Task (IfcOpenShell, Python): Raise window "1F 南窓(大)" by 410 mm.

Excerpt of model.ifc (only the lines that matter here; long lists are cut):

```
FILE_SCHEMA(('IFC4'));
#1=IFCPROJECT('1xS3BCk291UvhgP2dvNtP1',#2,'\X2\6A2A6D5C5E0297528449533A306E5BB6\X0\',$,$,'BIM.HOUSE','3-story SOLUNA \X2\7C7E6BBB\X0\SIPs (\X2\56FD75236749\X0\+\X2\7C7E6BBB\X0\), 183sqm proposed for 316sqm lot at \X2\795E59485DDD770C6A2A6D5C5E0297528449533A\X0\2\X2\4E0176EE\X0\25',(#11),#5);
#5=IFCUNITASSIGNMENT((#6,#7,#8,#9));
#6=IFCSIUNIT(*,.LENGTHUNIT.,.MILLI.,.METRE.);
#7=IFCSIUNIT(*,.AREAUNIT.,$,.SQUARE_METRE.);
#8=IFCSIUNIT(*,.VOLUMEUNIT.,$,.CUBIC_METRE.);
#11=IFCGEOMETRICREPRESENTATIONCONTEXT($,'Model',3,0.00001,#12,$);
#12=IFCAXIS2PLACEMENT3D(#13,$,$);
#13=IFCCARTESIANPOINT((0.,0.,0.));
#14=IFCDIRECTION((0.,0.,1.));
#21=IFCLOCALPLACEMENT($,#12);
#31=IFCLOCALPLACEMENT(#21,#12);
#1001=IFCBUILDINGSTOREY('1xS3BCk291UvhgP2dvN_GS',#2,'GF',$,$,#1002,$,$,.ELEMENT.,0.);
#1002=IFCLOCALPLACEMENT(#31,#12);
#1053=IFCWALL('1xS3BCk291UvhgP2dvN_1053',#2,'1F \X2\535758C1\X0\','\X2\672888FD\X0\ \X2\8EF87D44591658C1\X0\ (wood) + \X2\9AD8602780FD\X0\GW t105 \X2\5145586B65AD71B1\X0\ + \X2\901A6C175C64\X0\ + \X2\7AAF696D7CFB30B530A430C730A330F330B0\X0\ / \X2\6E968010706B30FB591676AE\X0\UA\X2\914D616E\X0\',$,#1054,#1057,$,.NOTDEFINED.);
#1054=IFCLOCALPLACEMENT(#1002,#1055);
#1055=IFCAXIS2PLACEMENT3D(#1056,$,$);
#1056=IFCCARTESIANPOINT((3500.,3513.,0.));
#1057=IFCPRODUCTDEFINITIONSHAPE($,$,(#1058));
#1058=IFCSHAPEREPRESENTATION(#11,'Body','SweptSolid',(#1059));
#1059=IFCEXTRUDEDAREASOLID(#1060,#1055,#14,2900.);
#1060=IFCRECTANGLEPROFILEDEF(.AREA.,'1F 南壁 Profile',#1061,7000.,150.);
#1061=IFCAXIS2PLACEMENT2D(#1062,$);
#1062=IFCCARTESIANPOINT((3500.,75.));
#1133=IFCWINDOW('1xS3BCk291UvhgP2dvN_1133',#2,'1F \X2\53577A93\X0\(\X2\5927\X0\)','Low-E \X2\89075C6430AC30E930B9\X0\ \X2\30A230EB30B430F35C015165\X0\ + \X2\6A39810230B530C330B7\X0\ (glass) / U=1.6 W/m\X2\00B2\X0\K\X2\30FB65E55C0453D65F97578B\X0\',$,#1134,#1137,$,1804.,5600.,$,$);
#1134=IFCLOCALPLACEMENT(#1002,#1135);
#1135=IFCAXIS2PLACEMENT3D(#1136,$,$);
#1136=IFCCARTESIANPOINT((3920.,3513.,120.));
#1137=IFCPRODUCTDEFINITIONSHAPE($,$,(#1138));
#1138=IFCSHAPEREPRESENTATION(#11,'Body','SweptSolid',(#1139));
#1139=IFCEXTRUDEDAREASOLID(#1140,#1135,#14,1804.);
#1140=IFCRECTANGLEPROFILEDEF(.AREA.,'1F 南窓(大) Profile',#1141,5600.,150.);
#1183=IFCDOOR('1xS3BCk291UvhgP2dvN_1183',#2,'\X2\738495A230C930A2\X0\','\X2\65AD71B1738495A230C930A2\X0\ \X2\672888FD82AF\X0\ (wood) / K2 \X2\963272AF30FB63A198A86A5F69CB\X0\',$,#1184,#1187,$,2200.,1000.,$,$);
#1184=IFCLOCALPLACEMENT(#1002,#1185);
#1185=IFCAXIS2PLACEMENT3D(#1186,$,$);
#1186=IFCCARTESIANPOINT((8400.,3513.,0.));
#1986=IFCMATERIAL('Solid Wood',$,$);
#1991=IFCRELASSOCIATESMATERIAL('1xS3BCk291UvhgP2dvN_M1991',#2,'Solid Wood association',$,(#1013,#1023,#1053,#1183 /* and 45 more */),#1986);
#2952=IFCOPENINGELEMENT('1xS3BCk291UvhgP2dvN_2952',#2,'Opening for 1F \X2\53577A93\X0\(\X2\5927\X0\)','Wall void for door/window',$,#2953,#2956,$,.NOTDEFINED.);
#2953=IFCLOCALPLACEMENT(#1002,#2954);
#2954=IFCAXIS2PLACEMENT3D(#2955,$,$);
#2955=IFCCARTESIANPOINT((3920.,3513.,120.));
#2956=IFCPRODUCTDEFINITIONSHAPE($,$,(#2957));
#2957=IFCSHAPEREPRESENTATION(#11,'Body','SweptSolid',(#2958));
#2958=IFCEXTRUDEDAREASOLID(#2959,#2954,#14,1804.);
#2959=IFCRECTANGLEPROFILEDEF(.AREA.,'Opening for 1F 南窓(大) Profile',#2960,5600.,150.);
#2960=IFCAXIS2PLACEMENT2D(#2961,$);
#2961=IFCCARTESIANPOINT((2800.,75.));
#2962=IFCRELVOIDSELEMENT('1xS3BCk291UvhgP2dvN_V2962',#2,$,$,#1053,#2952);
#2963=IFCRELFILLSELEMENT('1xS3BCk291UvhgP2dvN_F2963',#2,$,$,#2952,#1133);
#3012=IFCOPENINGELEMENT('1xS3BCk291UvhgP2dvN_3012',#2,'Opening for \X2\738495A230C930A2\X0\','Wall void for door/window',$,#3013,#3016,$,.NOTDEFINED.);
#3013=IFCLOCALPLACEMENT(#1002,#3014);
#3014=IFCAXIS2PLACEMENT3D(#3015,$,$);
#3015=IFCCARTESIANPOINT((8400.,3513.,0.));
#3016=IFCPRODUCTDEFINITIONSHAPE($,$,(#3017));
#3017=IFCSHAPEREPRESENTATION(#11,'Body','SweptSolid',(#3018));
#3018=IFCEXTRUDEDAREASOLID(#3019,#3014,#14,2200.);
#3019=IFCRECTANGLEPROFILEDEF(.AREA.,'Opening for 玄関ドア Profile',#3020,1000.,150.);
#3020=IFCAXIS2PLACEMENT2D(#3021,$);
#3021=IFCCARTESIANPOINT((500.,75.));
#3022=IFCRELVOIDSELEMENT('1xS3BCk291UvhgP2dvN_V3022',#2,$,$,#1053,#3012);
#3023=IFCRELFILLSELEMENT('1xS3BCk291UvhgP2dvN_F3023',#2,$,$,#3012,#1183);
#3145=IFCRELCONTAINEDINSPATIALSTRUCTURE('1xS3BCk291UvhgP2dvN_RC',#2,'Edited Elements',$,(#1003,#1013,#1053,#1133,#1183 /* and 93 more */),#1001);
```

```python
import numpy as np
import ifcopenshell
import ifcopenshell.api.geometry
import ifcopenshell.util.placement
import ifcopenshell.util.unit

model = ifcopenshell.open("model.ifc")
unit_scale = ifcopenshell.util.unit.calculate_unit_scale(model)

window = model.by_guid("1xS3BCk291UvhgP2dvN_1133")
opening = window.FillsVoids[0].RelatingOpeningElement
dz = 0.41 / unit_scale

shift = np.array([0.0, 0.0, dz])
# The window is not placed relative to its opening, so move both.
for product in (opening, window):
    matrix = ifcopenshell.util.placement.get_local_placement(product.ObjectPlacement)
    matrix[:3, 3] += shift
    ifcopenshell.api.geometry.edit_object_placement(model, product=product, matrix=matrix, is_si=False)

print(f"moved by {dz * unit_scale:+.3f} m")

model.write("model-out.ifc")
```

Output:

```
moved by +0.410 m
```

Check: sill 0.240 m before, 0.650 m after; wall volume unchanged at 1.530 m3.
